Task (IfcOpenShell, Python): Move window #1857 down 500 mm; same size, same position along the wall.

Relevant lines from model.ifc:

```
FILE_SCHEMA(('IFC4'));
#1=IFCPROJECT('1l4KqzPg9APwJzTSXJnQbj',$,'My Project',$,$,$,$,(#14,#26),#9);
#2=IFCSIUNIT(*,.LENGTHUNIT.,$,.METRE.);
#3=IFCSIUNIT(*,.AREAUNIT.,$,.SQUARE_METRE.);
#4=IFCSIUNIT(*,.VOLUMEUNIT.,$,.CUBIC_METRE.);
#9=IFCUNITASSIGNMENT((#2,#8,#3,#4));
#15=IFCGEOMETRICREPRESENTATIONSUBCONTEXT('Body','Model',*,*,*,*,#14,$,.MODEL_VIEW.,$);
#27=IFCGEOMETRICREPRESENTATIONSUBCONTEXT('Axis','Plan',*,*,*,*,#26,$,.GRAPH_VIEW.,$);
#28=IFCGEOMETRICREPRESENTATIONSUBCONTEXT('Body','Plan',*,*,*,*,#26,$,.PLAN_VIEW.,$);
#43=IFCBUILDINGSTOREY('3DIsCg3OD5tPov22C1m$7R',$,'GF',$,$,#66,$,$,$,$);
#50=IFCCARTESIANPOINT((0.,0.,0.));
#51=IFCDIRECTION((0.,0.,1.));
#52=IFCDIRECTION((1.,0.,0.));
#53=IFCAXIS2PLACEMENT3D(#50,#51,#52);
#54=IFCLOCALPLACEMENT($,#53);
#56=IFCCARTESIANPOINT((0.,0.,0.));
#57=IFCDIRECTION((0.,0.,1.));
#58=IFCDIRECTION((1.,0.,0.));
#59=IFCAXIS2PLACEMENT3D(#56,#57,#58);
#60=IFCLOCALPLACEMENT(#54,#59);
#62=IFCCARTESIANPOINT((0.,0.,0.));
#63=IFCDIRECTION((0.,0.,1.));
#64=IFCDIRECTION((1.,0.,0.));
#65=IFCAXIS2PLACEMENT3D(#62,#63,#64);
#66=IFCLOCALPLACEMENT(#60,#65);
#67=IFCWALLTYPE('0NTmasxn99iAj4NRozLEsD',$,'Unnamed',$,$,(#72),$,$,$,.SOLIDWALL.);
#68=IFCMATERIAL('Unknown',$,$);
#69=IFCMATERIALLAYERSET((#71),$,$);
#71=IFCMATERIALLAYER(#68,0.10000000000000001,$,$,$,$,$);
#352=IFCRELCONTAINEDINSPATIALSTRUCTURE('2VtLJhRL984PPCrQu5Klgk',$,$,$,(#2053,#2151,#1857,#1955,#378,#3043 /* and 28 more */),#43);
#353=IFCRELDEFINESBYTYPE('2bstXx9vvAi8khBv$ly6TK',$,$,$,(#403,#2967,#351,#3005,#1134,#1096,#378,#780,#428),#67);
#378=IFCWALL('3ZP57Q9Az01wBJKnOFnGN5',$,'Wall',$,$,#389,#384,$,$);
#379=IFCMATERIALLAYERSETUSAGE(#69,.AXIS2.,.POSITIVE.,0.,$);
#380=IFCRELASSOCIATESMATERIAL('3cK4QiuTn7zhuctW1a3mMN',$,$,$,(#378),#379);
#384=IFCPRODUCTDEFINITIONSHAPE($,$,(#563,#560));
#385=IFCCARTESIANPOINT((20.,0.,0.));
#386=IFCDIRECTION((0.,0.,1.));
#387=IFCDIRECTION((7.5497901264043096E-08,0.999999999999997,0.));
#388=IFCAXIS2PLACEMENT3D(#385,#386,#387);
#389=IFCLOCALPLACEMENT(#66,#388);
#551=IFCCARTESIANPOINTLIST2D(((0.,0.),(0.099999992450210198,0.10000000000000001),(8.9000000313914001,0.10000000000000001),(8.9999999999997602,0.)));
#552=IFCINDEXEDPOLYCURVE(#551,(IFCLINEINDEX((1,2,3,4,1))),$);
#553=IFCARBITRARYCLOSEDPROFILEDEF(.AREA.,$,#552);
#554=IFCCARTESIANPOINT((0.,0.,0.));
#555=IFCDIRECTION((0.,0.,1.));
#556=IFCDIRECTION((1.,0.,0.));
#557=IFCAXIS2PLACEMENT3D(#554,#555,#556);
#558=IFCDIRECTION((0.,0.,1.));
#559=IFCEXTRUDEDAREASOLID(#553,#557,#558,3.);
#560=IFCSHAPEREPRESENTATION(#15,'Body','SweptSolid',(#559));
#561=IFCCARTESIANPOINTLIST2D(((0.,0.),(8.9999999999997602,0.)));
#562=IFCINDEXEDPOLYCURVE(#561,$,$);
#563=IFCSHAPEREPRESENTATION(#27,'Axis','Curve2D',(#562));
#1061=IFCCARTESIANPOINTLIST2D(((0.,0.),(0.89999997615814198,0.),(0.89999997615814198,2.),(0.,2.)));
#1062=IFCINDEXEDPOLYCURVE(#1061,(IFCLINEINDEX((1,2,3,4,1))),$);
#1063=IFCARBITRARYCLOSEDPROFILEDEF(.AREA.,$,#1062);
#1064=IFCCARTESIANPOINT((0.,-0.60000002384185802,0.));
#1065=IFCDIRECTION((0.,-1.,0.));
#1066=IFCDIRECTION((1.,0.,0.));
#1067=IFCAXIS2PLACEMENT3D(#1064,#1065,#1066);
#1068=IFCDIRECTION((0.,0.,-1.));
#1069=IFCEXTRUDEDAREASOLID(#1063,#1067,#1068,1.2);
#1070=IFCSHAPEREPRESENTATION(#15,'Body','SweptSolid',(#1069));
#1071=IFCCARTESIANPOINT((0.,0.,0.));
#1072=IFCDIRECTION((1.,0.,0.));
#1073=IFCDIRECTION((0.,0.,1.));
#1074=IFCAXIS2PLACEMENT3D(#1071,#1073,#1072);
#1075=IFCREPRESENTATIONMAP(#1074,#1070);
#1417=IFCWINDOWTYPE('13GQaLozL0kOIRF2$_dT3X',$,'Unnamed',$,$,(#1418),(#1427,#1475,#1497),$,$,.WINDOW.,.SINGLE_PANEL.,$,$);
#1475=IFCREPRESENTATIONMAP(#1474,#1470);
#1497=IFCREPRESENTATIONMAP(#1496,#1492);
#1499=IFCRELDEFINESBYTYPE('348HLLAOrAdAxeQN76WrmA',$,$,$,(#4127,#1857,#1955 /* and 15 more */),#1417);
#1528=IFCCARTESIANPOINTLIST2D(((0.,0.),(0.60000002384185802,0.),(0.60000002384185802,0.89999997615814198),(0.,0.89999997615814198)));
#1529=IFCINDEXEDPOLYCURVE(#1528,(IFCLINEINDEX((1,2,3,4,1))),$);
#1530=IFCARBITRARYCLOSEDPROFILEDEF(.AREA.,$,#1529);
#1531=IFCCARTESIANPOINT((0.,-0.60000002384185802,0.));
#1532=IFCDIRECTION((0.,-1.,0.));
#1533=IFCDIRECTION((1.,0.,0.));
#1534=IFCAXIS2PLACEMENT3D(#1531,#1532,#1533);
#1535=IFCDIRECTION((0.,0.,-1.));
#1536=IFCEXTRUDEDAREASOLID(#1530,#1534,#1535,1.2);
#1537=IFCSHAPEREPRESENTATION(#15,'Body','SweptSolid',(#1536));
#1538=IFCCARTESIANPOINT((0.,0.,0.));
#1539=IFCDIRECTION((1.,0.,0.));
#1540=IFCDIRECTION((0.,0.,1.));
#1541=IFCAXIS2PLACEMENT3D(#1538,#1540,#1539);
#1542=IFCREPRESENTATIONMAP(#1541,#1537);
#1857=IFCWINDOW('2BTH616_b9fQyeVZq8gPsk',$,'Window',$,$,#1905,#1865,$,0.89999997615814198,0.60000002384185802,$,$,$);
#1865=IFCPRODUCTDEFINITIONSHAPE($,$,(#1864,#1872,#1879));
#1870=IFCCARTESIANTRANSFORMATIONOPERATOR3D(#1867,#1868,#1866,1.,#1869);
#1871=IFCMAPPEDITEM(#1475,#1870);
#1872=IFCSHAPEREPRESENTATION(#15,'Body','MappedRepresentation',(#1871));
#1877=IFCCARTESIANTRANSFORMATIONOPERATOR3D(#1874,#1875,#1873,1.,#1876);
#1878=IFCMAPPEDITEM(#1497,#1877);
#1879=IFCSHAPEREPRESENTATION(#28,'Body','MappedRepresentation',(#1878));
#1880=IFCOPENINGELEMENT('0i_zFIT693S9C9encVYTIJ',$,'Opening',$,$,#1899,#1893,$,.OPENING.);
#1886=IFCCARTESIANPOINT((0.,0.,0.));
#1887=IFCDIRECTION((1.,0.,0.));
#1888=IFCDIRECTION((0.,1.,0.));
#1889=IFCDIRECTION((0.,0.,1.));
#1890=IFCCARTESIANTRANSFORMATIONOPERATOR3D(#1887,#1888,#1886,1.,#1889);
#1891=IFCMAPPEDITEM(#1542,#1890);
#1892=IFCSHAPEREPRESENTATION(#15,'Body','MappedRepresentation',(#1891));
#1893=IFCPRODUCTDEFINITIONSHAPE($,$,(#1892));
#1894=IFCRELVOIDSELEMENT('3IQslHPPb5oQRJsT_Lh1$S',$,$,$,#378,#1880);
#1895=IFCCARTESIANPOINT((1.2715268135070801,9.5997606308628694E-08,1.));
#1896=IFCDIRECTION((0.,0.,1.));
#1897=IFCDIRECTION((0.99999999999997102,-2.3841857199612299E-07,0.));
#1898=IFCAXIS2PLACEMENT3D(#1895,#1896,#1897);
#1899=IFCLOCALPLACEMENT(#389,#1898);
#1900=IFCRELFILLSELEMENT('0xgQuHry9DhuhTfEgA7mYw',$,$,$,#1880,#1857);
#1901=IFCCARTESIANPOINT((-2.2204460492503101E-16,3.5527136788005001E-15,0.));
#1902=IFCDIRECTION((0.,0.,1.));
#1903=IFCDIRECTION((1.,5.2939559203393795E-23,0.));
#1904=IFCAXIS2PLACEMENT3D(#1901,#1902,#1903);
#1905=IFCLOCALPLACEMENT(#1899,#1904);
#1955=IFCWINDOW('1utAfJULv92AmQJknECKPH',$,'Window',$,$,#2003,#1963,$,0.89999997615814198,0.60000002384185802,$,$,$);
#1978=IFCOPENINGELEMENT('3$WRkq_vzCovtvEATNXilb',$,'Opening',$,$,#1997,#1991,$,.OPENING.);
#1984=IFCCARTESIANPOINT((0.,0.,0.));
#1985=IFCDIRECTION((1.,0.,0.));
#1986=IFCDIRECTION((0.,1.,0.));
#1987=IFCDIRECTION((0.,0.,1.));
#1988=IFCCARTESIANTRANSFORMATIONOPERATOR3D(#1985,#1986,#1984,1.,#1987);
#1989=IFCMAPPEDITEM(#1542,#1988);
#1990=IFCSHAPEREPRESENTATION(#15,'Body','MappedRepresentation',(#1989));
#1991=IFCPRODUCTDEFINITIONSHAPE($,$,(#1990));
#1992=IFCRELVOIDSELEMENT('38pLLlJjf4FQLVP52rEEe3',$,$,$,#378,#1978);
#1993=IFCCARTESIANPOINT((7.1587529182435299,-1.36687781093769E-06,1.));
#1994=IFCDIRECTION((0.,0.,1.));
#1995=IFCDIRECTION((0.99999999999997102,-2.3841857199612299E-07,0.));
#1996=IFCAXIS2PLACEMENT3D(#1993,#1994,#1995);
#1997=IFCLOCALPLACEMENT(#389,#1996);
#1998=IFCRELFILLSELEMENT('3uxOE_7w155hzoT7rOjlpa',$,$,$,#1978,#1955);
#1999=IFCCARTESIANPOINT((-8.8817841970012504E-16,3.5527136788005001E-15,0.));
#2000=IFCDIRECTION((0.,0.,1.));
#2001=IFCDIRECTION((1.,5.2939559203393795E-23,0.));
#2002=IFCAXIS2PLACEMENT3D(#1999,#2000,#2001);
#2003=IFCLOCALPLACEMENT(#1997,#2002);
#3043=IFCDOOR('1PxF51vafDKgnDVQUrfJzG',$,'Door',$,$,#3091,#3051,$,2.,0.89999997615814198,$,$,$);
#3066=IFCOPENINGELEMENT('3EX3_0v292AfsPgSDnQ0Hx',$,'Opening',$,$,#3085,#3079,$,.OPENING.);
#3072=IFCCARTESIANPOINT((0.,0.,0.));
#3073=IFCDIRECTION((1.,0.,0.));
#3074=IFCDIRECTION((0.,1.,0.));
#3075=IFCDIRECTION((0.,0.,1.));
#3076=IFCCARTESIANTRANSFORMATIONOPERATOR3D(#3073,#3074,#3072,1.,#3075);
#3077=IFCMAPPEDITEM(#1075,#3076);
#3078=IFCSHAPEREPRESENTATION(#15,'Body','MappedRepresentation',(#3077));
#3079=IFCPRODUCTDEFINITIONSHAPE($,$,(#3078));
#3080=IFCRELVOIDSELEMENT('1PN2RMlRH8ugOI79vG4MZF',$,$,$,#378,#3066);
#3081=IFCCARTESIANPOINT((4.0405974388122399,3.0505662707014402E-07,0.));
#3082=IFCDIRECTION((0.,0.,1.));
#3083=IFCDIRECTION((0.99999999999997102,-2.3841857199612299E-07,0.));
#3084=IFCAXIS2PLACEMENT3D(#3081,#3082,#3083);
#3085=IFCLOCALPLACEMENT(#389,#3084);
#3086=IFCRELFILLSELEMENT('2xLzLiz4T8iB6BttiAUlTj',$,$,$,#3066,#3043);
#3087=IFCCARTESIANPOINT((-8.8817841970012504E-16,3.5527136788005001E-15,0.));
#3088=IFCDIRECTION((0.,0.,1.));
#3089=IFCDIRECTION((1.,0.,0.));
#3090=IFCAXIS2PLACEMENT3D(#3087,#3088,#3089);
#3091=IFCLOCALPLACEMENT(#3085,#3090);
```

```python
import numpy as np
import ifcopenshell
import ifcopenshell.api.geometry
import ifcopenshell.util.placement
import ifcopenshell.util.unit

model = ifcopenshell.open("model.ifc")
unit_scale = ifcopenshell.util.unit.calculate_unit_scale(model)

window = model.by_guid("2BTH616_b9fQyeVZq8gPsk")
opening = window.FillsVoids[0].RelatingOpeningElement
dz = -0.5 / unit_scale

shift = np.array([0.0, 0.0, dz])
# The window is placed relative to its opening, so it follows when the opening moves.
matrix = ifcopenshell.util.placement.get_local_placement(opening.ObjectPlacement)
matrix[:3, 3] += shift
ifcopenshell.api.geometry.edit_object_placement(
    model, product=opening, matrix=matrix, is_si=False, should_transform_children=True
)

print(f"moved by {dz * unit_scale:+.3f} m")

model.write("model_v2.ifc")
```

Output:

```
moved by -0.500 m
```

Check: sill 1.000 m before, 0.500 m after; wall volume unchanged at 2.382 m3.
